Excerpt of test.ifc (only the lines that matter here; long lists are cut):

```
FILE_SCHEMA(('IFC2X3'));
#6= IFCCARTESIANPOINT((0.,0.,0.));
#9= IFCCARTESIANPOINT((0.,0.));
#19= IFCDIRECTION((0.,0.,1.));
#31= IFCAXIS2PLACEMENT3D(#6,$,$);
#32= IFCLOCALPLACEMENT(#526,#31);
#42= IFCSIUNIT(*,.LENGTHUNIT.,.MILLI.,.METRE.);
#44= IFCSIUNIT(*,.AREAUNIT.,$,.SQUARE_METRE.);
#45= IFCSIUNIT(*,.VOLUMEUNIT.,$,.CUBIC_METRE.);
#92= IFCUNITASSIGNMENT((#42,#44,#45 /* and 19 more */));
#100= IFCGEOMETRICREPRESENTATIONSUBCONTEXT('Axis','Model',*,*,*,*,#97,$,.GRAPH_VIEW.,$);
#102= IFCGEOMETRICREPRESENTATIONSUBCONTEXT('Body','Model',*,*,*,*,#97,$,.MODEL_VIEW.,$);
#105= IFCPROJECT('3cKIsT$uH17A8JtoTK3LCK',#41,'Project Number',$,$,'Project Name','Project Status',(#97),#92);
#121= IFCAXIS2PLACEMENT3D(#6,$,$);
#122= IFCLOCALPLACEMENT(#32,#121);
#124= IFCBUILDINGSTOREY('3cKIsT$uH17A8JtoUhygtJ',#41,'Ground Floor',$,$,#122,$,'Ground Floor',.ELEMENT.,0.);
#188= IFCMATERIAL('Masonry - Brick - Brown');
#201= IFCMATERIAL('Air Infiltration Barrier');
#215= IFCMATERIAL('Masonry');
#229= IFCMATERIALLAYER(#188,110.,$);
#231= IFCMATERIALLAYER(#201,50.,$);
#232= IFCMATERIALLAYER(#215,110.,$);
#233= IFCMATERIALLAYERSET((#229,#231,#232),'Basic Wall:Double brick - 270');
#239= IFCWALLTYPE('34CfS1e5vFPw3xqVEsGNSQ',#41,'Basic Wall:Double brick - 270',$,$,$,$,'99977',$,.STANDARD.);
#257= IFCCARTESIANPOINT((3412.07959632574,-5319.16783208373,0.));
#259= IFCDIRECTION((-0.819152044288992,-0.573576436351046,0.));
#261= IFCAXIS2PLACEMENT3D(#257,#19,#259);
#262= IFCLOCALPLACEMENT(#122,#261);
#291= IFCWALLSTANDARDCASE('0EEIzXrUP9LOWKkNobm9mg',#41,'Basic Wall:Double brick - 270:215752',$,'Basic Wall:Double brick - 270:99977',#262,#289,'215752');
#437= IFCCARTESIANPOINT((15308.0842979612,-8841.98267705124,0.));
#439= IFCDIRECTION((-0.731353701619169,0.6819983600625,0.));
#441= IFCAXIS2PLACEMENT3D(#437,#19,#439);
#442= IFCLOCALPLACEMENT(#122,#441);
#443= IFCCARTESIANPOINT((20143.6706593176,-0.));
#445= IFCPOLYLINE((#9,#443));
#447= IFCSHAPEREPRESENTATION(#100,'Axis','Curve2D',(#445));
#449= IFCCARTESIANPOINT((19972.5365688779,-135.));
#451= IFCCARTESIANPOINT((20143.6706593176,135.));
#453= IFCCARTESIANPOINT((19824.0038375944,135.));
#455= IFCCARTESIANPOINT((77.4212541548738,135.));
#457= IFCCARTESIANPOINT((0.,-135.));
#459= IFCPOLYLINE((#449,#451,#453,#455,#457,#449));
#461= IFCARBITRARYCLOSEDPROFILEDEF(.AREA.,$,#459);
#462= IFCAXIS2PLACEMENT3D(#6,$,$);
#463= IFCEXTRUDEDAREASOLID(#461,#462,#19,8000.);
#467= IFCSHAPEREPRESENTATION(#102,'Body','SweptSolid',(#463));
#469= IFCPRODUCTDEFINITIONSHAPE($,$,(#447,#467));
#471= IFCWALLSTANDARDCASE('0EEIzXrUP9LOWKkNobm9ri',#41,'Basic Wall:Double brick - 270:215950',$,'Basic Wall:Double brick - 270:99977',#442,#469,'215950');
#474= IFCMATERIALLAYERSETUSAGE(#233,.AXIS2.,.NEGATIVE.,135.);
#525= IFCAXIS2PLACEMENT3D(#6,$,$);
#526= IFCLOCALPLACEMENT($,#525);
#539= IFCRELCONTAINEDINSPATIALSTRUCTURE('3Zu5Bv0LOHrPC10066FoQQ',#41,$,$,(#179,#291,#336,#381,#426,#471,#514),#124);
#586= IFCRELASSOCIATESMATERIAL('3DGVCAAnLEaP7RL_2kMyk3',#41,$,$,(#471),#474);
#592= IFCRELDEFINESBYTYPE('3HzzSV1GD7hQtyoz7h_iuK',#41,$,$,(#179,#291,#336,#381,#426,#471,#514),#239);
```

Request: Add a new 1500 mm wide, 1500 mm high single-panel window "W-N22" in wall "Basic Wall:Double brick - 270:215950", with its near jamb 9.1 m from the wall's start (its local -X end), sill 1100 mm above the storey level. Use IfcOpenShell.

```python
import numpy as np
import ifcopenshell
import ifcopenshell.api.feature
import ifcopenshell.api.geometry
import ifcopenshell.api.root
import ifcopenshell.api.spatial
import ifcopenshell.api.type
import ifcopenshell.geom
import ifcopenshell.util.element
import ifcopenshell.util.placement
import ifcopenshell.util.representation
import ifcopenshell.util.shape
import ifcopenshell.util.unit

model = ifcopenshell.open("test.ifc")
unit_scale = ifcopenshell.util.unit.calculate_unit_scale(model)
settings = ifcopenshell.geom.settings()


def volume(element):
    """Net volume in cubic metres, openings subtracted."""
    shape = ifcopenshell.geom.create_shape(settings, element)
    return ifcopenshell.util.shape.get_volume(shape.geometry)


wall = model.by_id(471)
storey = ifcopenshell.util.element.get_container(wall, ifc_class="IfcBuildingStorey")
context = ifcopenshell.util.representation.get_context(model, "Model", "Body", "MODEL_VIEW")
before = volume(wall)

width, height, from_end, sill = 1.5, 1.5, 9.1, 1.1  # metres

# The wall runs along its own X axis, and the end named is its -X end.
wall_shape = ifcopenshell.geom.create_shape(settings, wall)
x, y, z = ifcopenshell.util.shape.get_vertices(wall_shape.geometry).T
start = x.min() + from_end
face, thickness = float(y.min()), float(y.max() - y.min())
wall_matrix = ifcopenshell.util.placement.get_local_placement(wall.ObjectPlacement)
level = ifcopenshell.util.placement.get_local_placement(storey.ObjectPlacement)[2, 3]


def in_wall(x, y):
    """Placement at x, y metres in the wall's axes, at sill height."""
    matrix = wall_matrix.copy()
    matrix[:, 3] = wall_matrix @ np.array([x / unit_scale, y / unit_scale, 0.0, 1.0])
    matrix[2, 3] = level + sill / unit_scale
    return matrix


# Opening: a box that overshoots both wall faces by 50 mm.
opening = ifcopenshell.api.root.create_entity(model, ifc_class="IfcOpeningElement")
box = ifcopenshell.api.geometry.add_wall_representation(
    model, context=context, length=width, height=height, thickness=thickness + 0.1
)
ifcopenshell.api.geometry.assign_representation(model, product=opening, representation=box)
ifcopenshell.api.geometry.edit_object_placement(model, product=opening, matrix=in_wall(start, face - 0.05), is_si=False)
ifcopenshell.api.feature.add_feature(model, feature=opening, element=wall)

window = ifcopenshell.api.root.create_entity(model, ifc_class="IfcWindow", name="W-N22")
window.OverallWidth, window.OverallHeight = width / unit_scale, height / unit_scale
body = ifcopenshell.api.geometry.add_window_representation(
    model,
    context=context,
    overall_width=window.OverallWidth,
    overall_height=window.OverallHeight,
    partition_type="SINGLE_PANEL",
)
ifcopenshell.api.geometry.assign_representation(model, product=window, representation=body)
ifcopenshell.api.spatial.assign_container(model, products=[window], relating_structure=storey)
fills = ifcopenshell.api.feature.add_filling(model, opening=opening, element=window)
fills.OwnerHistory = window.OwnerHistory  # required in IFC2X3

# IFC2X3 keeps the operation on the window style.
style = ifcopenshell.api.root.create_entity(model, ifc_class="IfcWindowStyle", name="W-N22")
style.OperationType, style.ConstructionType = "SINGLE_PANEL", "NOTDEFINED"
style.ParameterTakesPrecedence = style.Sizeable = False
ifcopenshell.api.type.assign_type(model, related_objects=[window], relating_type=style)

# Centre the window in the wall's thickness.
ifcopenshell.api.geometry.edit_object_placement(model, product=window, matrix=in_wall(start, face), is_si=False)
window_shape = ifcopenshell.geom.create_shape(settings, window)
depth = ifcopenshell.util.shape.get_vertices(window_shape.geometry)[:, 1]
offset = face + thickness / 2 - (depth.min() + depth.max()) / 2
ifcopenshell.api.geometry.edit_object_placement(model, product=window, matrix=in_wall(start, offset), is_si=False)

after = volume(wall)

print(f"wall volume {before:.3f} -> {after:.3f} m3")

model.write("test_v2.ifc")
```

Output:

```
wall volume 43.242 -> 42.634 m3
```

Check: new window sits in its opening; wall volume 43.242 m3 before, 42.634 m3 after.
